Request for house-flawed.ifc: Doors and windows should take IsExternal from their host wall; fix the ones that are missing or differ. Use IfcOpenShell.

First a look at what the model holds.

```python
import ifcopenshell
import ifcopenshell.util.element

model = ifcopenshell.open("house-flawed.ifc")
print(model.schema)
seen = {}
for e in model.by_type("IfcDoor") + model.by_type("IfcWindow"):
    if not e.FillsVoids:
        continue
    host = e.FillsVoids[0].RelatingOpeningElement.VoidsElements[0].RelatingBuildingElement
    own = ifcopenshell.util.element.get_pset(e, f"Pset_{e.is_a()[3:].removesuffix('StandardCase')}Common", "IsExternal")
    wall = ifcopenshell.util.element.get_pset(host, "Pset_WallCommon", "IsExternal")
    seen[e.is_a(), own, wall] = seen.get((e.is_a(), own, wall), 0) + 1
for (cls, own, wall), count in sorted(seen.items(), key=str):
    print(count, cls, "IsExternal:", own, "| host wall:", wall)
```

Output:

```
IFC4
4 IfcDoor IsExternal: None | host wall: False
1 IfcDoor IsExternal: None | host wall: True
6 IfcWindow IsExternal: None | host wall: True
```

```python
import ifcopenshell
import ifcopenshell.api.pset
import ifcopenshell.util.element

model = ifcopenshell.open("house-flawed.ifc")

count = 0
for ifc_class, pset_name in (("IfcDoor", "Pset_DoorCommon"), ("IfcWindow", "Pset_WindowCommon")):
    for e in model.by_type(ifc_class):
        if not e.FillsVoids:
            continue
        host = e.FillsVoids[0].RelatingOpeningElement.VoidsElements[0].RelatingBuildingElement
        external = ifcopenshell.util.element.get_pset(host, "Pset_WallCommon", "IsExternal")
        if external is None or ifcopenshell.util.element.get_pset(e, pset_name, "IsExternal") == external:
            continue
        pset = ifcopenshell.api.pset.add_pset(model, product=e, name=pset_name)
        ifcopenshell.api.pset.edit_pset(model, pset=pset, properties={"IsExternal": external})
        count += 1

print(count, "updated")

model.write("house-flawed_rev.ifc")
```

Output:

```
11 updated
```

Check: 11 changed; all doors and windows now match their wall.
